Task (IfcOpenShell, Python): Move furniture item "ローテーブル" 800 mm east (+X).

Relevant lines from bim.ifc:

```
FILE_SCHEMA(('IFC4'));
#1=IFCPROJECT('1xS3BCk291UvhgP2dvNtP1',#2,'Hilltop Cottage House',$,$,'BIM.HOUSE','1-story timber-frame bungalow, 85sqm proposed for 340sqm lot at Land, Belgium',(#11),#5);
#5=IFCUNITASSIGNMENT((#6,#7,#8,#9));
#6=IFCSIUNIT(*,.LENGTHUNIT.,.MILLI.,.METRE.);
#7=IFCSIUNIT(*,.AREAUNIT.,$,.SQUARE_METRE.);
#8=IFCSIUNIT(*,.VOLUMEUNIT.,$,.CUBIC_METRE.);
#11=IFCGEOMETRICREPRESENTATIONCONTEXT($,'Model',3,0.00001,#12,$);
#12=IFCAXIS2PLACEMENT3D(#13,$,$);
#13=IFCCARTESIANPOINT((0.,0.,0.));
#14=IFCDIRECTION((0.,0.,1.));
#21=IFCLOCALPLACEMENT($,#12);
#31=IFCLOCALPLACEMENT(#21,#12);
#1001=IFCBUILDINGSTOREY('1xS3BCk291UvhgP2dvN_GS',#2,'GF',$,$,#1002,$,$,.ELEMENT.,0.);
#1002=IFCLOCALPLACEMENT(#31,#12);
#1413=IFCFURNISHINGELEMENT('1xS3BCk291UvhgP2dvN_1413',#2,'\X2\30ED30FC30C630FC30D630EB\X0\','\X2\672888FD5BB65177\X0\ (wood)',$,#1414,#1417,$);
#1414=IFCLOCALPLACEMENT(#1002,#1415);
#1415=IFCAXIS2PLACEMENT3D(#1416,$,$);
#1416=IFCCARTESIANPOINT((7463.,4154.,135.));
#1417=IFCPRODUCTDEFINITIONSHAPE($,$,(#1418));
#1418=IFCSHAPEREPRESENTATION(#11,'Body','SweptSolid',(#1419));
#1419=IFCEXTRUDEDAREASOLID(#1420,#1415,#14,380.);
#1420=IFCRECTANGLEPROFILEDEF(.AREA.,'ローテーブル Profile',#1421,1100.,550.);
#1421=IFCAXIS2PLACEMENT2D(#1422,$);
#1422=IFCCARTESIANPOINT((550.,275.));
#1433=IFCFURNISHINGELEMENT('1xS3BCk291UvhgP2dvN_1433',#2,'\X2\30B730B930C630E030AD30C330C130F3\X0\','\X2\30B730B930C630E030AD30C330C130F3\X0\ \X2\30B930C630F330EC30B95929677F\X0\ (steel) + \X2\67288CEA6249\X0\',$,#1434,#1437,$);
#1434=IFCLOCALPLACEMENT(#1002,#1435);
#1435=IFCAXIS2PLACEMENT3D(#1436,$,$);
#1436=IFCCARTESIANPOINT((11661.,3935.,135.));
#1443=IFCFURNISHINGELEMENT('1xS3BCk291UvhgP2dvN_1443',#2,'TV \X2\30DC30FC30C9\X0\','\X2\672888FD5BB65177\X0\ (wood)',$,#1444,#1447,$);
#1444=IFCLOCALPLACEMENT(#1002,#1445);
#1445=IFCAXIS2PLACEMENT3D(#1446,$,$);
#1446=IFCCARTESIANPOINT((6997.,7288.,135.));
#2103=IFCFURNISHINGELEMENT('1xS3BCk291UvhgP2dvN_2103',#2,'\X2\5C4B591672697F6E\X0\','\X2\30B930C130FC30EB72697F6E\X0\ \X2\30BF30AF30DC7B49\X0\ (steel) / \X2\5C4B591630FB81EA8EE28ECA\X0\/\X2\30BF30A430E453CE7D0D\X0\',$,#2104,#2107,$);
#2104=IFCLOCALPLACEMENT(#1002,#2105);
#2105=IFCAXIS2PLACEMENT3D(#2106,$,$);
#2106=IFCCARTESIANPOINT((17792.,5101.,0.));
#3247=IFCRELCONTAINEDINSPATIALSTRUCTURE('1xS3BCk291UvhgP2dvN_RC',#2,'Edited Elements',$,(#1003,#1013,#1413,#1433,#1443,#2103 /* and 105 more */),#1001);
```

```python
import ifcopenshell
import ifcopenshell.api.geometry
import ifcopenshell.util.placement
import ifcopenshell.util.unit

model = ifcopenshell.open("bim.ifc")
unit_scale = ifcopenshell.util.unit.calculate_unit_scale(model)

item = model.by_guid("1xS3BCk291UvhgP2dvN_1413")
matrix = ifcopenshell.util.placement.get_local_placement(item.ObjectPlacement)
matrix[0, 3] += 0.8 / unit_scale
ifcopenshell.api.geometry.edit_object_placement(model, product=item, matrix=matrix, is_si=False)

print(ifcopenshell.util.placement.get_local_placement(item.ObjectPlacement).round(3) + 0.0)

model.write("bim_edited.ifc")
```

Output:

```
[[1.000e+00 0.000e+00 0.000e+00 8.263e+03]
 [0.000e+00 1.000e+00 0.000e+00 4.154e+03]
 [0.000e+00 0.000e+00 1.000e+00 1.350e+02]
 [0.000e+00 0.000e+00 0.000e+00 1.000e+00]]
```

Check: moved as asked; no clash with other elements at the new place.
